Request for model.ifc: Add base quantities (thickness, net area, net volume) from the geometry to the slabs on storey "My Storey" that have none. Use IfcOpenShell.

First a look at what the model holds.

```python
import ifcopenshell
import ifcopenshell.util.element
import ifcopenshell.util.unit

model = ifcopenshell.open("model.ifc")
print(model.schema)
for unit_type in ("LENGTHUNIT", "AREAUNIT", "VOLUMEUNIT"):
    print(unit_type, ifcopenshell.util.unit.calculate_unit_scale(model, unit_type))
storey = next(s for s in model.by_type("IfcBuildingStorey") if s.Name == "My Storey")
slabs = [e for e in ifcopenshell.util.element.get_decomposition(storey) if e.is_a("IfcSlab")]
for e in sorted(slabs, key=lambda e: e.id()):
    print(e.id(), e.is_a(), e.Name, list(ifcopenshell.util.element.get_psets(e, qtos_only=True)), sep=" | ")
```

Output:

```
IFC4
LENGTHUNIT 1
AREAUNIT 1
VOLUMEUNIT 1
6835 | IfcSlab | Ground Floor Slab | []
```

```python
import ifcopenshell
import ifcopenshell.api.pset
import ifcopenshell.geom
import ifcopenshell.util.element
import ifcopenshell.util.shape
import ifcopenshell.util.unit

model = ifcopenshell.open("model.ifc")
unit_scale = ifcopenshell.util.unit.calculate_unit_scale(model)
area_scale = ifcopenshell.util.unit.calculate_unit_scale(model, "AREAUNIT")
volume_scale = ifcopenshell.util.unit.calculate_unit_scale(model, "VOLUMEUNIT")
settings = ifcopenshell.geom.settings()

storey = next(s for s in model.by_type("IfcBuildingStorey") if s.Name == "My Storey")
slabs = [e for e in ifcopenshell.util.element.get_decomposition(storey) if e.is_a("IfcSlab")]

for e in sorted(slabs, key=lambda e: e.id()):
    if ifcopenshell.util.element.get_psets(e, qtos_only=True, should_inherit=False):
        continue
    # Geometry comes back in metres, in the element's own axes.
    shape = ifcopenshell.geom.create_shape(settings, e)
    values = {
        "Width": ifcopenshell.util.shape.get_z(shape.geometry) / unit_scale,
        "NetArea": ifcopenshell.util.shape.get_footprint_area(shape.geometry) / area_scale,
        "NetVolume": ifcopenshell.util.shape.get_volume(shape.geometry) / volume_scale,
    }
    qto = ifcopenshell.api.pset.add_qto(model, product=e, name="Qto_SlabBaseQuantities")
    ifcopenshell.api.pset.edit_qto(model, qto=qto, properties=values)
    print(e.id(), {k: round(v, 3) for k, v in values.items()})

model.write("model-out.ifc")
```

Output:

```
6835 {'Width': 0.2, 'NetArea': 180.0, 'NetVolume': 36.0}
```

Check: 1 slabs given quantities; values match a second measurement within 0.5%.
